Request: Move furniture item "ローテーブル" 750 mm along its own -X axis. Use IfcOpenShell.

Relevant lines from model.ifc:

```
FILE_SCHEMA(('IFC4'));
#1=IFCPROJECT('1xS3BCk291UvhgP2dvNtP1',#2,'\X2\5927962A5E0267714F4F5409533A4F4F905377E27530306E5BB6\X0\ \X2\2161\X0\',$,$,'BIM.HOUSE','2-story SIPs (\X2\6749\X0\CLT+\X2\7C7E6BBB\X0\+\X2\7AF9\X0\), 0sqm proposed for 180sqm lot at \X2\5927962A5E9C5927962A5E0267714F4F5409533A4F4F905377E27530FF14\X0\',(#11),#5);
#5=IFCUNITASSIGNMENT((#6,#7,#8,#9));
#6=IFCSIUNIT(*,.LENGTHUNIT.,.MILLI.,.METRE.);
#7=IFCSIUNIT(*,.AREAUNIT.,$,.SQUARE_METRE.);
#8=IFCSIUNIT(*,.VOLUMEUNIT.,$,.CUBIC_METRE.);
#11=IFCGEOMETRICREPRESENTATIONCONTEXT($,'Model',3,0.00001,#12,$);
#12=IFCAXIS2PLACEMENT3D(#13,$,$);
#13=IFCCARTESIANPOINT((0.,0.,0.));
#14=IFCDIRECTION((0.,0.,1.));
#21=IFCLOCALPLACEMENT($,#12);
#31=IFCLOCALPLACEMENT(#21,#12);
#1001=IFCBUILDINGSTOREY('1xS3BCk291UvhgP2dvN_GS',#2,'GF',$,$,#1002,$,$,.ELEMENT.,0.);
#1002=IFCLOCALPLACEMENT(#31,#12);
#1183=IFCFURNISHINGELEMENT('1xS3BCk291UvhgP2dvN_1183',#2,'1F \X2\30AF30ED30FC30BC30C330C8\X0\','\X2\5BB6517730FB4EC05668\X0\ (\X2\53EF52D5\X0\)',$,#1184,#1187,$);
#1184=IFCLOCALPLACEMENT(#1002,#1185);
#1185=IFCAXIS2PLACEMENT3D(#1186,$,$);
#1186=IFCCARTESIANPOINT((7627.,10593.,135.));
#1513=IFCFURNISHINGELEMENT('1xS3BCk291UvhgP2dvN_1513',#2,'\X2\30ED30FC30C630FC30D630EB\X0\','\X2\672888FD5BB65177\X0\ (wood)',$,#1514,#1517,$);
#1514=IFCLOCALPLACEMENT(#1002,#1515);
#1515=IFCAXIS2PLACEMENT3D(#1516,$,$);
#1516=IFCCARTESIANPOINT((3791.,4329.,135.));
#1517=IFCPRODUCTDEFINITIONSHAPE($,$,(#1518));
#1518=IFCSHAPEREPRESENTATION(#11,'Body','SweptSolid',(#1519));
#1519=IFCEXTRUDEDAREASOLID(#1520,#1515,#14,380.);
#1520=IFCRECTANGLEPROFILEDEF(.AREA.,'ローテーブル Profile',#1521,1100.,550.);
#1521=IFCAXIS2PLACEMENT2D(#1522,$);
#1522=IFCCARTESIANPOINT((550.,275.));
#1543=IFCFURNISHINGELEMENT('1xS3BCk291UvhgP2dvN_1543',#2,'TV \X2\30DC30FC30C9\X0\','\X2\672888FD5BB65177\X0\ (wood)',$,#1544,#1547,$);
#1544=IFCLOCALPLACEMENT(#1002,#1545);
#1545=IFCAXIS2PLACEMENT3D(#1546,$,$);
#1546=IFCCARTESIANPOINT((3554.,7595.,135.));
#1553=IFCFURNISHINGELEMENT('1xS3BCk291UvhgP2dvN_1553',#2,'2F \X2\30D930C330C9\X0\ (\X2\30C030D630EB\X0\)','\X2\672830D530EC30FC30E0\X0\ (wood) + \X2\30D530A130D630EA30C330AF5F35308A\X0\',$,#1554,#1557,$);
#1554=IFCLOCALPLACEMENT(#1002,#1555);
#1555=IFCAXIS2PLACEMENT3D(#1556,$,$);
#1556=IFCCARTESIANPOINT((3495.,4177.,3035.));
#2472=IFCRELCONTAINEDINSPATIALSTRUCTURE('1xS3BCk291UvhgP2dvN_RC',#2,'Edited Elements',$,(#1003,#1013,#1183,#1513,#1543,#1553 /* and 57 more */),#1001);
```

```python
import ifcopenshell
import ifcopenshell.api.geometry
import ifcopenshell.util.placement
import ifcopenshell.util.unit

model = ifcopenshell.open("model.ifc")
unit_scale = ifcopenshell.util.unit.calculate_unit_scale(model)

item = model.by_guid("1xS3BCk291UvhgP2dvN_1513")
matrix = ifcopenshell.util.placement.get_local_placement(item.ObjectPlacement)
matrix[:3, 3] -= matrix[:3, 0] * 0.75 / unit_scale
ifcopenshell.api.geometry.edit_object_placement(model, product=item, matrix=matrix, is_si=False)

print(ifcopenshell.util.placement.get_local_placement(item.ObjectPlacement).round(3) + 0.0)

model.write("model_updated.ifc")
```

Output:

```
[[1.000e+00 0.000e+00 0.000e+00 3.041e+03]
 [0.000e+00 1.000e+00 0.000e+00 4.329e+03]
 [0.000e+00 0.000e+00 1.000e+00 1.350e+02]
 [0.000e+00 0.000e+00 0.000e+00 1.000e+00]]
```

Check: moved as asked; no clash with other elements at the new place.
